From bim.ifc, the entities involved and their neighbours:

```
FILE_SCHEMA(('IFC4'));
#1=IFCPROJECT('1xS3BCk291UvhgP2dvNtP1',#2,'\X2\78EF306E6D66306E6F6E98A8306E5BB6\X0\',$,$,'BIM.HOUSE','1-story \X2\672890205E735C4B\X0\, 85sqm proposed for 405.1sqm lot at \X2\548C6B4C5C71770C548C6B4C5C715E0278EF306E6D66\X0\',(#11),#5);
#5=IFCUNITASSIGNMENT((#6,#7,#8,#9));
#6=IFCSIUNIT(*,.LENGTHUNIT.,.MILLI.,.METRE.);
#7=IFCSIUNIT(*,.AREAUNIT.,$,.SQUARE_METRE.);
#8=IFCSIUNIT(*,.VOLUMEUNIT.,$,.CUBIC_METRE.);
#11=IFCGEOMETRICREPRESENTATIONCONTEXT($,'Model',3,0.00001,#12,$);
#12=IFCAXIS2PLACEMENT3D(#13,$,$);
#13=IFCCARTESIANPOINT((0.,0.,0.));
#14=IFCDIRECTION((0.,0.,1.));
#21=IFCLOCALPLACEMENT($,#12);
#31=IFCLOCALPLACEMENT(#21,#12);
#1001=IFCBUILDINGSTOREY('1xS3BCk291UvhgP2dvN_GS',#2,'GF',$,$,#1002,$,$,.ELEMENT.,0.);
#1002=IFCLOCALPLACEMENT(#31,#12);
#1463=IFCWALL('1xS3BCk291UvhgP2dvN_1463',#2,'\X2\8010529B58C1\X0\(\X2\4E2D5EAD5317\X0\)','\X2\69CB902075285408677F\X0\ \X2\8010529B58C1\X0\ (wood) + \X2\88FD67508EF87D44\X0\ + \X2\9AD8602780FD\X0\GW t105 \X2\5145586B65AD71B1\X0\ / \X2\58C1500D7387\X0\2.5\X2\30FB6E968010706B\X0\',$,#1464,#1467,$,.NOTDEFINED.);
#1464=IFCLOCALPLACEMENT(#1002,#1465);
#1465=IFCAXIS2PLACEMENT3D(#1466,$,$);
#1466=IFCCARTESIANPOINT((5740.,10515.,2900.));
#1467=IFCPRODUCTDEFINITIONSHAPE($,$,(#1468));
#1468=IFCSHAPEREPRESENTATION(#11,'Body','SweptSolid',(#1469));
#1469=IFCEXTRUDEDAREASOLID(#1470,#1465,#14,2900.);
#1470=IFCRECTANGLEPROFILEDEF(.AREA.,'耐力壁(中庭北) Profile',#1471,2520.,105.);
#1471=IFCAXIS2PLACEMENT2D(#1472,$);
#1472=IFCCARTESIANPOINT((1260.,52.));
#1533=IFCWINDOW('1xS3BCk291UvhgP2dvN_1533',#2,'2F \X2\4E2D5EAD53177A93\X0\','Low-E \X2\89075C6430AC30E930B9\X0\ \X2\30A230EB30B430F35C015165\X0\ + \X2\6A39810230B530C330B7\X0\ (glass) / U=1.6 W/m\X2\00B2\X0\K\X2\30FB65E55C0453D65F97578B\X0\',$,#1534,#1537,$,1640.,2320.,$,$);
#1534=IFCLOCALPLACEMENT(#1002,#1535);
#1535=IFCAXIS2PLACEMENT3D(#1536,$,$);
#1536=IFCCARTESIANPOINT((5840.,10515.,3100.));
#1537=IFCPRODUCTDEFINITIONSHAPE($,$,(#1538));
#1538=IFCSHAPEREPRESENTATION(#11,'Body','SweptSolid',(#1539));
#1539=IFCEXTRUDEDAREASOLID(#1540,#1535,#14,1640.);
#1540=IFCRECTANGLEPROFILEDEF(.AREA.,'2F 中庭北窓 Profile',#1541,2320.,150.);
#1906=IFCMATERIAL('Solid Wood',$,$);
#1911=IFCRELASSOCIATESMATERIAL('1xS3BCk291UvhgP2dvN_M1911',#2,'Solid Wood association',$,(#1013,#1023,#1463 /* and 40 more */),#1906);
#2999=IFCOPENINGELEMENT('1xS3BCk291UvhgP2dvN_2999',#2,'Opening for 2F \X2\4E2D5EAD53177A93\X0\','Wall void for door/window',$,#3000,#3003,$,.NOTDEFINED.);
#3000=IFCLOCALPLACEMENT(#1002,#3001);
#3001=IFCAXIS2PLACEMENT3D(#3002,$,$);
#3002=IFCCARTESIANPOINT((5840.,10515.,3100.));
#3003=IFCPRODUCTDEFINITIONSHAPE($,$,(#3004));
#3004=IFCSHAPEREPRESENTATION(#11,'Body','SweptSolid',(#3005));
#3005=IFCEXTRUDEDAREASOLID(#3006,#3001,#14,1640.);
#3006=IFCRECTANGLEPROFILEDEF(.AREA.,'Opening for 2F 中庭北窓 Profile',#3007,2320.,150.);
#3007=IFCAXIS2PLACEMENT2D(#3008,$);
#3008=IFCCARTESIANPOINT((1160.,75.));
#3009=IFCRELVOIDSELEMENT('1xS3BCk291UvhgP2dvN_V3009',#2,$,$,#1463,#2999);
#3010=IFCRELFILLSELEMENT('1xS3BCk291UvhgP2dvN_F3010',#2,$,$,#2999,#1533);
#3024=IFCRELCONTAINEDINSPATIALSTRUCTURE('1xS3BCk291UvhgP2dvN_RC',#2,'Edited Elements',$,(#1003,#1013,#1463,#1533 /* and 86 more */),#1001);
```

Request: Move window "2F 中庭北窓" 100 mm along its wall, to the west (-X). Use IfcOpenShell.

```python
import ifcopenshell
import ifcopenshell.api.geometry
import ifcopenshell.util.placement
import ifcopenshell.util.unit

model = ifcopenshell.open("bim.ifc")
unit_scale = ifcopenshell.util.unit.calculate_unit_scale(model)

window = model.by_guid("1xS3BCk291UvhgP2dvN_1533")
opening = window.FillsVoids[0].RelatingOpeningElement
wall = opening.VoidsElements[0].RelatingBuildingElement

wall_matrix = ifcopenshell.util.placement.get_local_placement(wall.ObjectPlacement)
shift = wall_matrix[:3, 0] * -0.1 / unit_scale
before = ifcopenshell.util.placement.get_local_placement(window.ObjectPlacement)[:3, 3].copy()

# The window is not placed relative to its opening, so move both.
for product in (opening, window):
    matrix = ifcopenshell.util.placement.get_local_placement(product.ObjectPlacement)
    matrix[:3, 3] += shift
    ifcopenshell.api.geometry.edit_object_placement(model, product=product, matrix=matrix, is_si=False)

after = ifcopenshell.util.placement.get_local_placement(window.ObjectPlacement)[:3, 3]
print("window moved by", (after - before).round(3) + 0.0)

model.write("bim_edited.ifc")
```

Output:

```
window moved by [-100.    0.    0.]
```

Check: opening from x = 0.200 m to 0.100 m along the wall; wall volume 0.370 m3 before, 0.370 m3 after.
